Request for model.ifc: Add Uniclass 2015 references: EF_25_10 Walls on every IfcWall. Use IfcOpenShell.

First a look at what the model holds.

```python
import ifcopenshell

model = ifcopenshell.open("model.ifc")
print(model.schema)
print("classifications:", [c.Name for c in model.by_type("IfcClassification")])
for ifc_class in ("IfcDoor", "IfcRoof", "IfcStair", "IfcWall", "IfcWindow"):
    print(ifc_class, len(model.by_type(ifc_class)))
```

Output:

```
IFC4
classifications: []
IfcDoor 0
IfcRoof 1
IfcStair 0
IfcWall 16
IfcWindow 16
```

```python
import ifcopenshell
import ifcopenshell.api.classification

model = ifcopenshell.open("model.ifc")

system = ifcopenshell.api.classification.add_classification(model, classification="Uniclass 2015")

codes = {
    "IfcWall": ("EF_25_10", "Walls"),
}
for ifc_class, (code, name) in codes.items():
    products = model.by_type(ifc_class)
    ifcopenshell.api.classification.add_reference(
        model, products=products, classification=system, identification=code, name=name
    )
    print(code, len(products))

model.write("model_rev.ifc")
```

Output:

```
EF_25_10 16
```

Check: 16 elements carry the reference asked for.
